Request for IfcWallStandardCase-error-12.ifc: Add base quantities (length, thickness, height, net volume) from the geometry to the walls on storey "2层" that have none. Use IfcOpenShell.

First a look at what the model holds.

```python
import ifcopenshell
import ifcopenshell.util.element
import ifcopenshell.util.unit

model = ifcopenshell.open("IfcWallStandardCase-error-12.ifc")
print(model.schema)
for unit_type in ("LENGTHUNIT", "AREAUNIT", "VOLUMEUNIT"):
    print(unit_type, ifcopenshell.util.unit.calculate_unit_scale(model, unit_type))
storey = next(s for s in model.by_type("IfcBuildingStorey") if s.Name == "2层")
walls = [e for e in ifcopenshell.util.element.get_decomposition(storey) if e.is_a("IfcWall")]
for e in sorted(walls, key=lambda e: e.id()):
    print(e.id(), e.is_a(), e.Name, list(ifcopenshell.util.element.get_psets(e, qtos_only=True)), sep=" | ")
```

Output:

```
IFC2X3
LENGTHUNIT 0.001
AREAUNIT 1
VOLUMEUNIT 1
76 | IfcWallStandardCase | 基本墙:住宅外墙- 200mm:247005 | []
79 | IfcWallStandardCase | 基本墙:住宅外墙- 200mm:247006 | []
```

```python
import ifcopenshell
import ifcopenshell.api.pset
import ifcopenshell.geom
import ifcopenshell.util.element
import ifcopenshell.util.shape
import ifcopenshell.util.unit

model = ifcopenshell.open("IfcWallStandardCase-error-12.ifc")
unit_scale = ifcopenshell.util.unit.calculate_unit_scale(model)
volume_scale = ifcopenshell.util.unit.calculate_unit_scale(model, "VOLUMEUNIT")
settings = ifcopenshell.geom.settings()

storey = next(s for s in model.by_type("IfcBuildingStorey") if s.Name == "2层")
walls = [e for e in ifcopenshell.util.element.get_decomposition(storey) if e.is_a("IfcWall")]

for e in sorted(walls, key=lambda e: e.id()):
    if ifcopenshell.util.element.get_psets(e, qtos_only=True, should_inherit=False):
        continue
    # Geometry comes back in metres, in the element's own axes.
    shape = ifcopenshell.geom.create_shape(settings, e)
    values = {
        "Length": ifcopenshell.util.shape.get_x(shape.geometry) / unit_scale,
        "Width": ifcopenshell.util.shape.get_y(shape.geometry) / unit_scale,
        "Height": ifcopenshell.util.shape.get_z(shape.geometry) / unit_scale,
        "NetVolume": ifcopenshell.util.shape.get_volume(shape.geometry) / volume_scale,
    }
    qto = ifcopenshell.api.pset.add_qto(model, product=e, name="BaseQuantities")
    ifcopenshell.api.pset.edit_qto(model, qto=qto, properties=values)
    print(e.id(), {k: round(v, 3) for k, v in values.items()})

model.write("IfcWallStandardCase-error-12_edited.ifc")
```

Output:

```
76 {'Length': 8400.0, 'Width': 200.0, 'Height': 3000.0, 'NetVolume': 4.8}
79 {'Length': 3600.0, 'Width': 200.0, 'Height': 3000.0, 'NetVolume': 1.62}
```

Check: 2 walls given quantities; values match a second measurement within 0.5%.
